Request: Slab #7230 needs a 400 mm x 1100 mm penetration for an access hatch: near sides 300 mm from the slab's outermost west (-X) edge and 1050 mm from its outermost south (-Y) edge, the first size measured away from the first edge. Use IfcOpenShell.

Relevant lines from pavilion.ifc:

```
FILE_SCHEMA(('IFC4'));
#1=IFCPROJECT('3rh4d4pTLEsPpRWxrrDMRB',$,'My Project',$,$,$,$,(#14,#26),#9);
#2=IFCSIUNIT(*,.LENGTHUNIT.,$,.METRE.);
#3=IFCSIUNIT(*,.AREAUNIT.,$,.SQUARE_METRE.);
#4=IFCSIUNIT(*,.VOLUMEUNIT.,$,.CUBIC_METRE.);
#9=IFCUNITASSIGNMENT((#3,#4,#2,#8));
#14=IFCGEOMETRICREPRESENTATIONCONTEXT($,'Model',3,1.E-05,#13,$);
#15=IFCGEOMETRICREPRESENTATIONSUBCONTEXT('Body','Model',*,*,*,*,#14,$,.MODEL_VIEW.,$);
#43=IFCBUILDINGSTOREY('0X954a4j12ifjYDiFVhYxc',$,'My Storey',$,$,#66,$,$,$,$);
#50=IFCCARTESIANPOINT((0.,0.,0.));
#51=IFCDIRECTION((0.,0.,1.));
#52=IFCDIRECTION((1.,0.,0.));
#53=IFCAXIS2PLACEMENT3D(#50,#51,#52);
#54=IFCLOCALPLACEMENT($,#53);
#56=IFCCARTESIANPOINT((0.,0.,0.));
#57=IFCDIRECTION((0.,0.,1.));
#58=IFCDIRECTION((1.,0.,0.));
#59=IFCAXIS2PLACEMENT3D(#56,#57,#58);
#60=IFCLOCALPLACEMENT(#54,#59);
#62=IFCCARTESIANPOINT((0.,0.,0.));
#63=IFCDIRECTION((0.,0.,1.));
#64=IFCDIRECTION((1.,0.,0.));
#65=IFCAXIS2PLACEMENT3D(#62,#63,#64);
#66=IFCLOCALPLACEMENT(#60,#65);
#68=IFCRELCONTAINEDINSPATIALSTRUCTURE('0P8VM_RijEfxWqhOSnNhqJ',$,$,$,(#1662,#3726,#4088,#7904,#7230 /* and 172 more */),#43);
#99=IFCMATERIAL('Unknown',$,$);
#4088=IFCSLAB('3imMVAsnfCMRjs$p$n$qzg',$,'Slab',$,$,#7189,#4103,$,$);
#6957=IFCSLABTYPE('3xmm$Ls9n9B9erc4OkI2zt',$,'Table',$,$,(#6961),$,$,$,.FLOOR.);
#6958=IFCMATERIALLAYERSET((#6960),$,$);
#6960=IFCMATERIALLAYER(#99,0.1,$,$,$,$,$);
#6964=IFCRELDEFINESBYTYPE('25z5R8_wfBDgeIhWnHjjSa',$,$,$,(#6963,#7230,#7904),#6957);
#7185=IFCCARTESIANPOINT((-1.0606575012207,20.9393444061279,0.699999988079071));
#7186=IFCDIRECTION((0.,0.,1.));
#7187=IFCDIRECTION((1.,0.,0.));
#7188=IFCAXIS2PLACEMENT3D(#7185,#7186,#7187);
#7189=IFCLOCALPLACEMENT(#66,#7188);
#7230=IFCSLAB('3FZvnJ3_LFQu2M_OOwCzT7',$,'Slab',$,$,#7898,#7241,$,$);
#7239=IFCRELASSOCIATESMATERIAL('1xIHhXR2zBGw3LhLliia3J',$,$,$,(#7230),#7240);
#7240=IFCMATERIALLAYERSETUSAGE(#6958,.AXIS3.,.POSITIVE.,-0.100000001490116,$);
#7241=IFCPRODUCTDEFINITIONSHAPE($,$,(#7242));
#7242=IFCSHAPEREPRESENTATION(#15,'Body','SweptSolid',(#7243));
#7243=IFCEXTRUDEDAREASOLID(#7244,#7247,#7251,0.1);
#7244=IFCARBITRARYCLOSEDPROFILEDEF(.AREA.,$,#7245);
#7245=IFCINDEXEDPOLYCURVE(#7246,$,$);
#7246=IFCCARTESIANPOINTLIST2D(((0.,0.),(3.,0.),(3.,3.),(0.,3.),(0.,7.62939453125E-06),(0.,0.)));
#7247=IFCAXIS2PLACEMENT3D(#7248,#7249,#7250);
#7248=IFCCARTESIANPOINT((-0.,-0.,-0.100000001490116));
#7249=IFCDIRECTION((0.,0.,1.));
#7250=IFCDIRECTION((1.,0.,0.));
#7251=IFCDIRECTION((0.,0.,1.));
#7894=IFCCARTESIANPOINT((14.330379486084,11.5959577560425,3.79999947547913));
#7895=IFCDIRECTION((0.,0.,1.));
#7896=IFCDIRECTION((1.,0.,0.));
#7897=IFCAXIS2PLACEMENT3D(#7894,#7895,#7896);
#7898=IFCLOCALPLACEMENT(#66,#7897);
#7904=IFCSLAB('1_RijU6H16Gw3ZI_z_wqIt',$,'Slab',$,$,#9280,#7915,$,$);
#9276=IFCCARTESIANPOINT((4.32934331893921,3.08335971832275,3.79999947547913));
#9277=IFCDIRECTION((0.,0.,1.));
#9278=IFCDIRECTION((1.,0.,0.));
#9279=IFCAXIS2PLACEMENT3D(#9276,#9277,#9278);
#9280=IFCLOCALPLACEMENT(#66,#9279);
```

```python
import numpy as np
import ifcopenshell
import ifcopenshell.api.feature
import ifcopenshell.api.geometry
import ifcopenshell.api.root
import ifcopenshell.geom
import ifcopenshell.util.placement
import ifcopenshell.util.representation
import ifcopenshell.util.shape
import ifcopenshell.util.unit

model = ifcopenshell.open("pavilion.ifc")
unit_scale = ifcopenshell.util.unit.calculate_unit_scale(model)
settings = ifcopenshell.geom.settings()


def volume(element):
    """Net volume in cubic metres, openings subtracted."""
    shape = ifcopenshell.geom.create_shape(settings, element)
    return ifcopenshell.util.shape.get_volume(shape.geometry)


slab = model.by_guid("3FZvnJ3_LFQu2M_OOwCzT7")
before = volume(slab)

# Extent in the slab's own axes, in metres. The edges named are its -X and -Y sides.
slab_shape = ifcopenshell.geom.create_shape(settings, slab)
vertices = ifcopenshell.util.shape.get_vertices(slab_shape.geometry)
x_min, y_min, bottom = vertices.min(axis=0)
top = vertices[:, 2].max()

opening = ifcopenshell.api.root.create_entity(model, ifc_class="IfcOpeningElement", name="Access hatch opening", predefined_type="OPENING")
context = ifcopenshell.util.representation.get_context(model, "Model", "Body", "MODEL_VIEW")
width, depth = 0.4, 1.1
outline = [(0.0, 0.0), (width, 0.0), (width, depth), (0.0, depth), (0.0, 0.0)]
# Overshoot both faces by 50 mm so the cut is clean.
shape = ifcopenshell.api.geometry.add_slab_representation(
    model, context=context, depth=top - bottom + 0.1, polyline=outline
)
ifcopenshell.api.geometry.assign_representation(model, product=opening, representation=shape)

matrix = ifcopenshell.util.placement.get_local_placement(slab.ObjectPlacement)
matrix[:, 3] = matrix @ np.append(np.array([x_min + 0.3, y_min + 1.05, bottom - 0.05]) / unit_scale, 1.0)
ifcopenshell.api.geometry.edit_object_placement(model, product=opening, matrix=matrix, is_si=False)
ifcopenshell.api.feature.add_feature(model, feature=opening, element=slab)

after = volume(slab)

print(f"slab volume {before:.3f} -> {after:.3f} m3")

model.write("pavilion_edited.ifc")
```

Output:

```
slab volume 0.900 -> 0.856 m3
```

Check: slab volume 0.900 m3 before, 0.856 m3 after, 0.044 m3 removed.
